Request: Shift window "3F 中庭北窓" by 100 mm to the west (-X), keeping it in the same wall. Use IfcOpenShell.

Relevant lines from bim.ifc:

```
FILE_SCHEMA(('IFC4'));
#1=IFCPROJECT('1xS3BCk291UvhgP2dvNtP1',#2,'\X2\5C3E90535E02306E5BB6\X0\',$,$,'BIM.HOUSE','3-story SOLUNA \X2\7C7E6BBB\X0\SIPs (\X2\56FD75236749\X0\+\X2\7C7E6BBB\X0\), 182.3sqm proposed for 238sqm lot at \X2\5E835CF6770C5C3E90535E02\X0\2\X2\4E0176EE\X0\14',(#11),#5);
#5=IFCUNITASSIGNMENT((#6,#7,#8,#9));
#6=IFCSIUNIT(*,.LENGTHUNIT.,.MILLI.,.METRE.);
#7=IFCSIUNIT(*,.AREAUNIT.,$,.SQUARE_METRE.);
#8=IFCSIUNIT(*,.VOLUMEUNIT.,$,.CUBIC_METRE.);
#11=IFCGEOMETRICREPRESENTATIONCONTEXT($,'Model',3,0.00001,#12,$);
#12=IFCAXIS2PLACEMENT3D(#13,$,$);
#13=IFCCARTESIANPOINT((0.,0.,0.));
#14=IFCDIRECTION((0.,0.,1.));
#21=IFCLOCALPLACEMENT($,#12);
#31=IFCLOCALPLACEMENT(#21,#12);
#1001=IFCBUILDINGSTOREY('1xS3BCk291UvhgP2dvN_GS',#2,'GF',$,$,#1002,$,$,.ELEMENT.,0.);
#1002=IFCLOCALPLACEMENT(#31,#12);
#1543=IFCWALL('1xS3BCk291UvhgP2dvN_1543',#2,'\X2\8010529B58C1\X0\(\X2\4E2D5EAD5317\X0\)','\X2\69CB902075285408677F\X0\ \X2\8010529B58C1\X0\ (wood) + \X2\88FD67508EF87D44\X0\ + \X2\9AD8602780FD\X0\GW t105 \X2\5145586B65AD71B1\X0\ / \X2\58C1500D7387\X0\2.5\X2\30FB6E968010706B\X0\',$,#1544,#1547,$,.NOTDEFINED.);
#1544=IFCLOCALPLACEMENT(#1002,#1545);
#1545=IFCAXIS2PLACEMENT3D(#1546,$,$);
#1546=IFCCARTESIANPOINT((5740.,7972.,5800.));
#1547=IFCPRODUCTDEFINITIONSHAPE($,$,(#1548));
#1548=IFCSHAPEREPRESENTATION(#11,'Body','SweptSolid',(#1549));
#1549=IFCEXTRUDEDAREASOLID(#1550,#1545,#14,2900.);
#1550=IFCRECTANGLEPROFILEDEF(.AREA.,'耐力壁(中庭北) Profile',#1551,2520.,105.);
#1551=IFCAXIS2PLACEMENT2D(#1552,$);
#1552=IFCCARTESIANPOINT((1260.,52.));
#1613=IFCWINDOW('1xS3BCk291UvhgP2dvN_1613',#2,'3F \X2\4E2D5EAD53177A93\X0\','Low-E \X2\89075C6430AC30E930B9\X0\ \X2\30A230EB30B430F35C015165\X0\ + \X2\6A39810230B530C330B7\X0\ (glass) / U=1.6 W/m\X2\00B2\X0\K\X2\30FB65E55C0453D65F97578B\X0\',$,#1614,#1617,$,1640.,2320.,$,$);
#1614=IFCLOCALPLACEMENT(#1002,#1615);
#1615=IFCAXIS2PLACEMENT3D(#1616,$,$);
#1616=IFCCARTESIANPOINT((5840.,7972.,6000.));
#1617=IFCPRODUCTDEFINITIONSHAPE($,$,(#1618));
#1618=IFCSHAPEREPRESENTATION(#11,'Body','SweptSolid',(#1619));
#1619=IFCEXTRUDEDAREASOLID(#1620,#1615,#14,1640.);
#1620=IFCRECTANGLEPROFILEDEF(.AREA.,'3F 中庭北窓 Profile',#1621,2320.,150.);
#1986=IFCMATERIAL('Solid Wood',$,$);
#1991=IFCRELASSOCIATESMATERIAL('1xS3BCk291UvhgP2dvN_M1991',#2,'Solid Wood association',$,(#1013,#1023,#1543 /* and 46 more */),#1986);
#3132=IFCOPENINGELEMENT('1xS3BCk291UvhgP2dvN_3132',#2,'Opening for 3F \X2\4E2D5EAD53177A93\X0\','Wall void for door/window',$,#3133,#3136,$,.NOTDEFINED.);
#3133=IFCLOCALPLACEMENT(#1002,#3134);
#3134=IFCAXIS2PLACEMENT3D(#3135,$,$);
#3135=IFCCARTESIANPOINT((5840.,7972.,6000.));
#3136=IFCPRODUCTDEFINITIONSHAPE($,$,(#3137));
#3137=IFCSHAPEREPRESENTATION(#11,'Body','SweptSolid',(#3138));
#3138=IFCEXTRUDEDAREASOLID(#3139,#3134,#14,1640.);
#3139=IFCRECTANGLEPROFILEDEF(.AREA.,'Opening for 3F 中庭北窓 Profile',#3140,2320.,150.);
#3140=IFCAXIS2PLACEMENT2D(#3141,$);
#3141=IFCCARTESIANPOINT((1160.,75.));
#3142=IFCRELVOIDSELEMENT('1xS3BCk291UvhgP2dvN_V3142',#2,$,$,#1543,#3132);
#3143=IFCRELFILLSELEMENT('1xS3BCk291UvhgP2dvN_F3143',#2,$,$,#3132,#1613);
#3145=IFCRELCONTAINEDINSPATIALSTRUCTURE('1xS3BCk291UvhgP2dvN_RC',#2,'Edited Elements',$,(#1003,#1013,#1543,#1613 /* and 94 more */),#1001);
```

```python
import ifcopenshell
import ifcopenshell.api.geometry
import ifcopenshell.util.placement
import ifcopenshell.util.unit

model = ifcopenshell.open("bim.ifc")
unit_scale = ifcopenshell.util.unit.calculate_unit_scale(model)

window = model.by_guid("1xS3BCk291UvhgP2dvN_1613")
opening = window.FillsVoids[0].RelatingOpeningElement
wall = opening.VoidsElements[0].RelatingBuildingElement

wall_matrix = ifcopenshell.util.placement.get_local_placement(wall.ObjectPlacement)
shift = wall_matrix[:3, 0] * -0.1 / unit_scale
before = ifcopenshell.util.placement.get_local_placement(window.ObjectPlacement)[:3, 3].copy()

# The window is not placed relative to its opening, so move both.
for product in (opening, window):
    matrix = ifcopenshell.util.placement.get_local_placement(product.ObjectPlacement)
    matrix[:3, 3] += shift
    ifcopenshell.api.geometry.edit_object_placement(model, product=product, matrix=matrix, is_si=False)

after = ifcopenshell.util.placement.get_local_placement(window.ObjectPlacement)[:3, 3]
print("window moved by", (after - before).round(3) + 0.0)

model.write("bim_updated.ifc")
```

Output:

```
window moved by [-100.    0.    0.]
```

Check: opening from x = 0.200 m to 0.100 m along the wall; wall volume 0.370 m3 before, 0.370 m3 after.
